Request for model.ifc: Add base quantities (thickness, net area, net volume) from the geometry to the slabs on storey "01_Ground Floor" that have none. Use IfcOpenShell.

First a look at what the model holds.

```python
import ifcopenshell
import ifcopenshell.util.element
import ifcopenshell.util.unit

model = ifcopenshell.open("model.ifc")
print(model.schema)
for unit_type in ("LENGTHUNIT", "AREAUNIT", "VOLUMEUNIT"):
    print(unit_type, ifcopenshell.util.unit.calculate_unit_scale(model, unit_type))
storey = next(s for s in model.by_type("IfcBuildingStorey") if s.Name == "01_Ground Floor")
slabs = [e for e in ifcopenshell.util.element.get_decomposition(storey) if e.is_a("IfcSlab")]
for e in sorted(slabs, key=lambda e: e.id()):
    print(e.id(), e.is_a(), e.Name, list(ifcopenshell.util.element.get_psets(e, qtos_only=True)), sep=" | ")
```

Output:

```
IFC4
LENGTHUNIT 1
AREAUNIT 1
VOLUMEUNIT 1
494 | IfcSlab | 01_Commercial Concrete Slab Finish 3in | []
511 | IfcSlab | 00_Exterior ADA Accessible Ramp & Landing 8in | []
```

```python
import ifcopenshell
import ifcopenshell.api.pset
import ifcopenshell.geom
import ifcopenshell.util.element
import ifcopenshell.util.shape
import ifcopenshell.util.unit

model = ifcopenshell.open("model.ifc")
unit_scale = ifcopenshell.util.unit.calculate_unit_scale(model)
area_scale = ifcopenshell.util.unit.calculate_unit_scale(model, "AREAUNIT")
volume_scale = ifcopenshell.util.unit.calculate_unit_scale(model, "VOLUMEUNIT")
settings = ifcopenshell.geom.settings()

storey = next(s for s in model.by_type("IfcBuildingStorey") if s.Name == "01_Ground Floor")
slabs = [e for e in ifcopenshell.util.element.get_decomposition(storey) if e.is_a("IfcSlab")]

for e in sorted(slabs, key=lambda e: e.id()):
    if ifcopenshell.util.element.get_psets(e, qtos_only=True, should_inherit=False):
        continue
    # Geometry comes back in metres, in the element's own axes.
    shape = ifcopenshell.geom.create_shape(settings, e)
    values = {
        "Width": ifcopenshell.util.shape.get_z(shape.geometry) / unit_scale,
        "NetArea": ifcopenshell.util.shape.get_footprint_area(shape.geometry) / area_scale,
        "NetVolume": ifcopenshell.util.shape.get_volume(shape.geometry) / volume_scale,
    }
    qto = ifcopenshell.api.pset.add_qto(model, product=e, name="Qto_SlabBaseQuantities")
    ifcopenshell.api.pset.edit_qto(model, qto=qto, properties=values)
    print(e.id(), {k: round(v, 3) for k, v in values.items()})

model.write("model-out.ifc")
```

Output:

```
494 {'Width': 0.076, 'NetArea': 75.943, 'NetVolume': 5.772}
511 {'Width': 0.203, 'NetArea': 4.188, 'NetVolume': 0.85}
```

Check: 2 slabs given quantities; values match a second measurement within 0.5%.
